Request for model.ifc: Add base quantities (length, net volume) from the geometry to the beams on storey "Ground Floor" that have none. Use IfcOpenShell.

First a look at what the model holds.

```python
import ifcopenshell
import ifcopenshell.util.element
import ifcopenshell.util.unit

model = ifcopenshell.open("model.ifc")
print(model.schema)
for unit_type in ("LENGTHUNIT", "AREAUNIT", "VOLUMEUNIT"):
    print(unit_type, ifcopenshell.util.unit.calculate_unit_scale(model, unit_type))
storey = next(s for s in model.by_type("IfcBuildingStorey") if s.Name == "Ground Floor")
beams = [e for e in ifcopenshell.util.element.get_decomposition(storey) if e.is_a("IfcBeam")]
for e in sorted(beams, key=lambda e: e.id()):
    print(e.id(), e.is_a(), e.Name, list(ifcopenshell.util.element.get_psets(e, qtos_only=True)), sep=" | ")
```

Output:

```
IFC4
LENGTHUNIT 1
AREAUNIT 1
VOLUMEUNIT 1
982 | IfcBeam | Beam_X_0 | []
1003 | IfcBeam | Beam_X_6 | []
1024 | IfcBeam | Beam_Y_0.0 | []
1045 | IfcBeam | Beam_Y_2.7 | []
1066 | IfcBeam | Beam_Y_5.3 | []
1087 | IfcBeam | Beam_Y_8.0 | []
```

```python
import ifcopenshell
import ifcopenshell.api.pset
import ifcopenshell.geom
import ifcopenshell.util.element
import ifcopenshell.util.shape
import ifcopenshell.util.unit

model = ifcopenshell.open("model.ifc")
unit_scale = ifcopenshell.util.unit.calculate_unit_scale(model)
volume_scale = ifcopenshell.util.unit.calculate_unit_scale(model, "VOLUMEUNIT")
settings = ifcopenshell.geom.settings()

storey = next(s for s in model.by_type("IfcBuildingStorey") if s.Name == "Ground Floor")
beams = [e for e in ifcopenshell.util.element.get_decomposition(storey) if e.is_a("IfcBeam")]

for e in sorted(beams, key=lambda e: e.id()):
    if ifcopenshell.util.element.get_psets(e, qtos_only=True, should_inherit=False):
        continue
    # Geometry comes back in metres, in the element's own axes.
    shape = ifcopenshell.geom.create_shape(settings, e)
    values = {
        "Length": ifcopenshell.util.shape.get_max_xyz(shape.geometry) / unit_scale,
        "NetVolume": ifcopenshell.util.shape.get_volume(shape.geometry) / volume_scale,
    }
    qto = ifcopenshell.api.pset.add_qto(model, product=e, name="Qto_BeamBaseQuantities")
    ifcopenshell.api.pset.edit_qto(model, qto=qto, properties=values)
    print(e.id(), {k: round(v, 3) for k, v in values.items()})

model.write("model_edited.ifc")
```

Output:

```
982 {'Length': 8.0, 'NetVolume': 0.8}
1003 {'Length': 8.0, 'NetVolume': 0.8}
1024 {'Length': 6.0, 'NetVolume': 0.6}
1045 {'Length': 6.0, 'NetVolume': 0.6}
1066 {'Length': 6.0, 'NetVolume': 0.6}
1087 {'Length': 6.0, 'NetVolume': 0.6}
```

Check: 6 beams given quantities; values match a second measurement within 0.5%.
